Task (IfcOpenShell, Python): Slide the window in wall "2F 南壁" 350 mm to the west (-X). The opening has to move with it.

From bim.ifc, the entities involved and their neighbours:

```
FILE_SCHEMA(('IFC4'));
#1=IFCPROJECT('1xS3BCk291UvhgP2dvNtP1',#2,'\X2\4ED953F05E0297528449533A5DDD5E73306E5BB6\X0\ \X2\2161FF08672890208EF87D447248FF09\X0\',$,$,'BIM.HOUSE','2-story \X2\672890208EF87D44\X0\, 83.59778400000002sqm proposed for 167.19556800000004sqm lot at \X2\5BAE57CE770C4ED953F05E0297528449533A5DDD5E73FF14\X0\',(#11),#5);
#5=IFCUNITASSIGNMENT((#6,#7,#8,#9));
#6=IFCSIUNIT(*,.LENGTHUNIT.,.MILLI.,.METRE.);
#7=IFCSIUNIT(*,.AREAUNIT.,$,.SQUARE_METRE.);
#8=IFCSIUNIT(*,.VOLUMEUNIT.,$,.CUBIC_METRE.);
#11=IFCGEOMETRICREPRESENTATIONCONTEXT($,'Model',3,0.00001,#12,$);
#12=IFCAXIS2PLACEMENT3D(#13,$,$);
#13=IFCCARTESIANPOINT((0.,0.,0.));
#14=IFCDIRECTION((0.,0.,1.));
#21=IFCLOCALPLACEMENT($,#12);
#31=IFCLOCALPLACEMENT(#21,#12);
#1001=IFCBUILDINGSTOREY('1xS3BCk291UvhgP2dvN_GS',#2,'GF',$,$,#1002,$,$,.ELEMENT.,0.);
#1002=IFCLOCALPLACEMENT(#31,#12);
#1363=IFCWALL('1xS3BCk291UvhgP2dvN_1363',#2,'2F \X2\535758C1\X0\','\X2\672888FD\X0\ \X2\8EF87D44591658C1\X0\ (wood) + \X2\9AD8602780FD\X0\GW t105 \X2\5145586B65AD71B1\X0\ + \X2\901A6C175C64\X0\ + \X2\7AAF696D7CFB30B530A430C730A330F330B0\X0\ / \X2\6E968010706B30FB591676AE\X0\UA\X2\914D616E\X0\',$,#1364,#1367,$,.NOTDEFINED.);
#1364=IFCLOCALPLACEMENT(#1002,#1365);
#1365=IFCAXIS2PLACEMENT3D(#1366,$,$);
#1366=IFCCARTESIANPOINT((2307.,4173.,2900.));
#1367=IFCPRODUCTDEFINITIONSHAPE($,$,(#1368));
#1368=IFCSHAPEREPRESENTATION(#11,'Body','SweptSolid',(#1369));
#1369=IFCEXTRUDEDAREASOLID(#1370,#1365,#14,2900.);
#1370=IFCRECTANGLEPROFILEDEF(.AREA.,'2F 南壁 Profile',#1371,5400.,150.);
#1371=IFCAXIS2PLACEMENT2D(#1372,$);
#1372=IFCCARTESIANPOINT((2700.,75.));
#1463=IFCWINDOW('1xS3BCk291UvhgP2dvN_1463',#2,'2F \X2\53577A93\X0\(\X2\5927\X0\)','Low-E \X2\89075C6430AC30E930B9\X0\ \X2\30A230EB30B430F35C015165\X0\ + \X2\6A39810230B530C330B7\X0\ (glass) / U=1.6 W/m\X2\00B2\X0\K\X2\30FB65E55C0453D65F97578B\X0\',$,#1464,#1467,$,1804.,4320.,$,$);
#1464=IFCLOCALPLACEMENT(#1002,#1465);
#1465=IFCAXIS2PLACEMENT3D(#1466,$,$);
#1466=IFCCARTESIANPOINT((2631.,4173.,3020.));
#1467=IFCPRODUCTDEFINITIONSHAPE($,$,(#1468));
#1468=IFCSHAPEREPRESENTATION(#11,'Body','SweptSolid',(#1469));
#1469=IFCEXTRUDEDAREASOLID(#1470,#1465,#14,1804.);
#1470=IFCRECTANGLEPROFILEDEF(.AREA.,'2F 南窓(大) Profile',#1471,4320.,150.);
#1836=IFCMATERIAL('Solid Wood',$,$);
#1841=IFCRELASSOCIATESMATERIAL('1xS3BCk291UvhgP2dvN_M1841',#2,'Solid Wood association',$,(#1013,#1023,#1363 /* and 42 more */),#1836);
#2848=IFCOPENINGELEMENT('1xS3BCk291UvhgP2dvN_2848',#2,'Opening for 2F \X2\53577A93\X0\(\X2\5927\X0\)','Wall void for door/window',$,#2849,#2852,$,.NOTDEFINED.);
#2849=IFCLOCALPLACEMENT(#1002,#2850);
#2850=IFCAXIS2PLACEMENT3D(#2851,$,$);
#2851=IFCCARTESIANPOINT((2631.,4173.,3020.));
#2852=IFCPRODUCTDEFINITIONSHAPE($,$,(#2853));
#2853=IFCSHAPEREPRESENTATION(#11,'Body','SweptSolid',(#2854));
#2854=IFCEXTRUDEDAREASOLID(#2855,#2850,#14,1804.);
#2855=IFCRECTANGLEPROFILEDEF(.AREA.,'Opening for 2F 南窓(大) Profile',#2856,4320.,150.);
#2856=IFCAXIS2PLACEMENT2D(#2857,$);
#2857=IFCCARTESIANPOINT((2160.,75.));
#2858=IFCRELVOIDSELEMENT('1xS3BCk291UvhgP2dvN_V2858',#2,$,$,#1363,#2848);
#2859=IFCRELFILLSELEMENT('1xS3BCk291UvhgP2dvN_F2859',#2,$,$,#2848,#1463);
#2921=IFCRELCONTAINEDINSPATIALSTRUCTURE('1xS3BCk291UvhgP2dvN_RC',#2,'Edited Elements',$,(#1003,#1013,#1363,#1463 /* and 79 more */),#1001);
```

```python
import ifcopenshell
import ifcopenshell.api.geometry
import ifcopenshell.util.placement
import ifcopenshell.util.unit

model = ifcopenshell.open("bim.ifc")
unit_scale = ifcopenshell.util.unit.calculate_unit_scale(model)

window = model.by_id(1463)
opening = window.FillsVoids[0].RelatingOpeningElement
wall = opening.VoidsElements[0].RelatingBuildingElement

wall_matrix = ifcopenshell.util.placement.get_local_placement(wall.ObjectPlacement)
shift = wall_matrix[:3, 0] * -0.35 / unit_scale
before = ifcopenshell.util.placement.get_local_placement(window.ObjectPlacement)[:3, 3].copy()

# The window is not placed relative to its opening, so move both.
for product in (opening, window):
    matrix = ifcopenshell.util.placement.get_local_placement(product.ObjectPlacement)
    matrix[:3, 3] += shift
    ifcopenshell.api.geometry.edit_object_placement(model, product=product, matrix=matrix, is_si=False)

after = ifcopenshell.util.placement.get_local_placement(window.ObjectPlacement)[:3, 3]
print("window moved by", (after - before).round(3) + 0.0)

model.write("bim_v2.ifc")
```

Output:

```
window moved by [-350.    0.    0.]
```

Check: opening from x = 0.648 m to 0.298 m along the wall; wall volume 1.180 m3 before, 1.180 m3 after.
